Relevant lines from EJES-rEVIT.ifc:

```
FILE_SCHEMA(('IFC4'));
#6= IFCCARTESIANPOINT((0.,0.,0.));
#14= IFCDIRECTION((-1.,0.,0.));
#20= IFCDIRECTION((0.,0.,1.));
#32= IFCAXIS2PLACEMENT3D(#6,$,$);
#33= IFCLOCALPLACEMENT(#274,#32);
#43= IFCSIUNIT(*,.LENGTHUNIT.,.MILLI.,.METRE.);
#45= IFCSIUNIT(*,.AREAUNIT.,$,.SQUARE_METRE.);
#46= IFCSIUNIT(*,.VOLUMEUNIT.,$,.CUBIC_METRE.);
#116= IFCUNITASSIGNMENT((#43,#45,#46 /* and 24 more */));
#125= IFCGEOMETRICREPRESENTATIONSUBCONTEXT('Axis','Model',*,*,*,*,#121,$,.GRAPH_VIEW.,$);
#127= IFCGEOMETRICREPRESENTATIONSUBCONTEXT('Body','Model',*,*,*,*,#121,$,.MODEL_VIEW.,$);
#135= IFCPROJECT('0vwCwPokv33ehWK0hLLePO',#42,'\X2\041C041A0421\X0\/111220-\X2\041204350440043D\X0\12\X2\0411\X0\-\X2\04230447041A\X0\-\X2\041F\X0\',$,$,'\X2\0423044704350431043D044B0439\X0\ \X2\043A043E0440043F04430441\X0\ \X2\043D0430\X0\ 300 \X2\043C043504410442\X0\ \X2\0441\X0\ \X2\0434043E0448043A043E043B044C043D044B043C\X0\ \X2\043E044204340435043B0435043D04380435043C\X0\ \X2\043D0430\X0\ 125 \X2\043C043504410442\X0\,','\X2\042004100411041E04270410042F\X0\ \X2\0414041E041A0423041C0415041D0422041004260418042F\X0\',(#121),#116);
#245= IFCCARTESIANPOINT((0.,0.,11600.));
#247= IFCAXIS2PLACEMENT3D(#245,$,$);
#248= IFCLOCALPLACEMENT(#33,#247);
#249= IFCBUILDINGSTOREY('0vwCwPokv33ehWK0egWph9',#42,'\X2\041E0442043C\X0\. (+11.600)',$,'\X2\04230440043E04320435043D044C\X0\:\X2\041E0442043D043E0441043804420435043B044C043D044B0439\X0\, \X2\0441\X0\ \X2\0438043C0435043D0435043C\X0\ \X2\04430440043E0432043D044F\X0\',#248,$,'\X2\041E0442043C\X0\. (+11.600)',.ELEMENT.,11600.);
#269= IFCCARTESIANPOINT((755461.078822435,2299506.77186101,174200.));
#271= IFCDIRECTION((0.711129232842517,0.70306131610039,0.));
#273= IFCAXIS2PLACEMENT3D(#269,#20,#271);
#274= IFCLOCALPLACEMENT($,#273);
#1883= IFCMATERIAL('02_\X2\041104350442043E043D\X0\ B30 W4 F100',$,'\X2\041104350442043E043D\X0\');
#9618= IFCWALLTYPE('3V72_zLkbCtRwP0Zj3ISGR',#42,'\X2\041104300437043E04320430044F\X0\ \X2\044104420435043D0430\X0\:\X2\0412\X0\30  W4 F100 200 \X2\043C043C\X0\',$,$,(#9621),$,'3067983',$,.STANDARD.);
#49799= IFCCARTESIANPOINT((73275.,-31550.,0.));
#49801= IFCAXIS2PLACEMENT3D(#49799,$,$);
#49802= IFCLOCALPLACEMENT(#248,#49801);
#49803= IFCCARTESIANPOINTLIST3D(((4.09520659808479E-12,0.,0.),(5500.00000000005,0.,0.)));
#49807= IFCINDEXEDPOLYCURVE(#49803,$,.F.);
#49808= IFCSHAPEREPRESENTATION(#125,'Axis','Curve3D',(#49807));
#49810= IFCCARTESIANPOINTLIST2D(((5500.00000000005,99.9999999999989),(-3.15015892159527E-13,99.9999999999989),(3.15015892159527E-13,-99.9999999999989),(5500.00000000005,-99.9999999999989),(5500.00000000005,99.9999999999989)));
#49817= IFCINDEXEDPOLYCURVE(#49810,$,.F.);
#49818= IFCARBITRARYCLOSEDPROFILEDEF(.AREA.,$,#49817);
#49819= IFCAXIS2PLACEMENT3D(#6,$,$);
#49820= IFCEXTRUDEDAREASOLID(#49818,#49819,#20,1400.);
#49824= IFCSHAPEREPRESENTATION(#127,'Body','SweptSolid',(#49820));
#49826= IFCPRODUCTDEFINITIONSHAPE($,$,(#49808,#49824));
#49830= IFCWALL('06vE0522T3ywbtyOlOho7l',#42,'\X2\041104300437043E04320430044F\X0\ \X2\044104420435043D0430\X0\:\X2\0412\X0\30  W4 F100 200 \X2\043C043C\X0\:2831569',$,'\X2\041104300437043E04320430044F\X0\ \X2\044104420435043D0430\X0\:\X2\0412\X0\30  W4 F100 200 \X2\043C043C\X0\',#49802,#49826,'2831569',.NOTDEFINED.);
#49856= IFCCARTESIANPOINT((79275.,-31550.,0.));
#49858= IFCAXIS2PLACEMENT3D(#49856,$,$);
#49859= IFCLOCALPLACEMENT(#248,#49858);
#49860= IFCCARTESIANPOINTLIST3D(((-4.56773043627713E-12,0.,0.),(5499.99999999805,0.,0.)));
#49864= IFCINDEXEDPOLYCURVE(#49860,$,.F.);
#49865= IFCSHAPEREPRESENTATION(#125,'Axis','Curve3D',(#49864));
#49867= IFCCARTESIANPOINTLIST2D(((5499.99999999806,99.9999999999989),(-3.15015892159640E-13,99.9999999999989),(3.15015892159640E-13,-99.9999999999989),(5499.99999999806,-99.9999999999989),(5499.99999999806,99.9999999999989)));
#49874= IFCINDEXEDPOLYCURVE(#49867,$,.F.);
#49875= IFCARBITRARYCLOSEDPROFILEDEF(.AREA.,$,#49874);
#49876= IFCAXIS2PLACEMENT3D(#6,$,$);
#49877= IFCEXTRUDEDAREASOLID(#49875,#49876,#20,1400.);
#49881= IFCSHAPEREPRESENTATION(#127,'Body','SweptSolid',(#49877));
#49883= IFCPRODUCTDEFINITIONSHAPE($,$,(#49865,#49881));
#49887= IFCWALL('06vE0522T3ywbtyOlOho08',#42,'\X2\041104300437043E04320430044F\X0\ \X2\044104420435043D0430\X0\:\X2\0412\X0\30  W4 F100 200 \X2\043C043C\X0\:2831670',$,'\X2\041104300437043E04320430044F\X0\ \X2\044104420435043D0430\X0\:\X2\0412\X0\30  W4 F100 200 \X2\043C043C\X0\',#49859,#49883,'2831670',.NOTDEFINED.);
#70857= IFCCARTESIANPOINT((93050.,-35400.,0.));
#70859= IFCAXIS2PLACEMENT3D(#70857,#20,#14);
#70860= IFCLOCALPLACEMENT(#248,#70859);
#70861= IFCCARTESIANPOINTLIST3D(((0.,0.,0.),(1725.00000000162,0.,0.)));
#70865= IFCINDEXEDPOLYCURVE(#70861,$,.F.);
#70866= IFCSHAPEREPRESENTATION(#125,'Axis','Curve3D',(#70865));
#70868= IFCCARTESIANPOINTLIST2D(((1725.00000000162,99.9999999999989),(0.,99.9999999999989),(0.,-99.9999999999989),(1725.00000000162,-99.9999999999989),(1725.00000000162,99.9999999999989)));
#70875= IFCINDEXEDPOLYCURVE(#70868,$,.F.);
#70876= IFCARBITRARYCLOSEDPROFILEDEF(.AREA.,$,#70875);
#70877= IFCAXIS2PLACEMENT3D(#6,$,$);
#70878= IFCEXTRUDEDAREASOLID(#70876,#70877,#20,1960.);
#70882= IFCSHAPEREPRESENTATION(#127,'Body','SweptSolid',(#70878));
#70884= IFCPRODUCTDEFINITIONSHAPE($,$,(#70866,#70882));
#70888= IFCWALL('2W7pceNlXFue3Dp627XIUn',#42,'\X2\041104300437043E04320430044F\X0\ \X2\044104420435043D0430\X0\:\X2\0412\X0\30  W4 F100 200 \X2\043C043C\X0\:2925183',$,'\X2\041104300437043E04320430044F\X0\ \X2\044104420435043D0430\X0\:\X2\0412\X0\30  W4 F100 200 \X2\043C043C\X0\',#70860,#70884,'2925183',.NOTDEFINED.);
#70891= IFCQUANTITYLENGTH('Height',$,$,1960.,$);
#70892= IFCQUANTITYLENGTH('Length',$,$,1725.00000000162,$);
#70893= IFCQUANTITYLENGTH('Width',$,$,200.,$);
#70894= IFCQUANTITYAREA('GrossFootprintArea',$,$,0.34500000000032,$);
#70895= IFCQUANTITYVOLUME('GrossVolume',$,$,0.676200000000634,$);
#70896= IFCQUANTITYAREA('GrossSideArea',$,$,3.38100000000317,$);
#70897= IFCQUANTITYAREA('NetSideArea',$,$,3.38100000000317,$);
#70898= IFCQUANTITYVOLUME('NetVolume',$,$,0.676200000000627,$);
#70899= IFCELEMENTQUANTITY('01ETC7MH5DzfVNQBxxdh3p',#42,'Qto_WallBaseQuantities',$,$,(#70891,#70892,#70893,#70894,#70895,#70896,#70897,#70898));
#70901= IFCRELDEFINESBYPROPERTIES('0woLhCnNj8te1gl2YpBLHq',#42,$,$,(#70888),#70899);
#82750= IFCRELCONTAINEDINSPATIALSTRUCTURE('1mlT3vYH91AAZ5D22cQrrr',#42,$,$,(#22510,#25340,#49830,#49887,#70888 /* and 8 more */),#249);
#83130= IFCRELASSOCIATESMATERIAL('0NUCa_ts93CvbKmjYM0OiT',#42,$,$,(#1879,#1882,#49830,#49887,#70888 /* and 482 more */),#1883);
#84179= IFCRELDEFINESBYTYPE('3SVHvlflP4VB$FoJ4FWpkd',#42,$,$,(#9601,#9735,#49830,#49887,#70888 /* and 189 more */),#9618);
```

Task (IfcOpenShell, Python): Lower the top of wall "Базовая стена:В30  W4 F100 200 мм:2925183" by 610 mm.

```python
import ifcopenshell
import ifcopenshell.api.pset
import ifcopenshell.geom
import ifcopenshell.util.element
import ifcopenshell.util.representation
import ifcopenshell.util.shape
import ifcopenshell.util.unit

model = ifcopenshell.open("EJES-rEVIT.ifc")
unit_scale = ifcopenshell.util.unit.calculate_unit_scale(model)
area_scale = ifcopenshell.util.unit.calculate_unit_scale(model, "AREAUNIT")
volume_scale = ifcopenshell.util.unit.calculate_unit_scale(model, "VOLUMEUNIT")
settings = ifcopenshell.geom.settings()


def volume(element):
    """Net volume in cubic metres, openings subtracted."""
    shape = ifcopenshell.geom.create_shape(settings, element)
    return ifcopenshell.util.shape.get_volume(shape.geometry)


wall = model.by_guid("2W7pceNlXFue3Dp627XIUn")
before = volume(wall)

body = ifcopenshell.util.representation.get_representation(wall, "Model", "Body")
solid = body.Items[0]
old_height = solid.Depth
solid.Depth -= 0.61 / unit_scale
after = volume(wall)
thickness = 0.2  # wall thickness in metres

# Update the stored height, areas and volumes.
qto = model.by_id(ifcopenshell.util.element.get_pset(wall, "Qto_WallBaseQuantities", should_inherit=False)["id"])
ifcopenshell.api.pset.edit_qto(model, qto=qto, properties={
    "Height": solid.Depth,
    "GrossVolume": ifcopenshell.util.element.get_pset(wall, "Qto_WallBaseQuantities", "GrossVolume") * solid.Depth / old_height,
    "GrossSideArea": ifcopenshell.util.element.get_pset(wall, "Qto_WallBaseQuantities", "GrossSideArea") * solid.Depth / old_height,
    "NetSideArea": after / thickness / area_scale,
    "NetVolume": after / volume_scale,
})

print(f"height {old_height:g} -> {solid.Depth:g}, volume {before:.3f} -> {after:.3f} m3")

model.write("EJES-rEVIT_updated.ifc")
```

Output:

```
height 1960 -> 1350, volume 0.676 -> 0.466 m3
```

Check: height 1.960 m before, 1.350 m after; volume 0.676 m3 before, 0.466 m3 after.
